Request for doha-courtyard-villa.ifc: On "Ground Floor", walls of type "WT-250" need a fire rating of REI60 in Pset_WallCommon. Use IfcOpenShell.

First a look at what the model holds.

```python
import ifcopenshell
import ifcopenshell.util.element

model = ifcopenshell.open("doha-courtyard-villa.ifc")
print(model.schema)
storey = next(s for s in model.by_type("IfcBuildingStorey") if s.Name == "Ground Floor")
walls = [e for e in ifcopenshell.util.element.get_decomposition(storey) if e.is_a("IfcWall")]
seen = {}
for e in walls:
    element_type = ifcopenshell.util.element.get_type(e)
    key = (element_type.Name if element_type != e and element_type else None, ifcopenshell.util.element.get_pset(e, "Pset_WallCommon", "FireRating"))
    seen[key] = seen.get(key, 0) + 1
for (name, value), count in sorted(seen.items(), key=str):
    print(count, "x", name, "|", value)
```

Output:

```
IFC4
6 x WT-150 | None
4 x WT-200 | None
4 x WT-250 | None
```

```python
import ifcopenshell
import ifcopenshell.api.pset
import ifcopenshell.util.element

model = ifcopenshell.open("doha-courtyard-villa.ifc")

storey = next(s for s in model.by_type("IfcBuildingStorey") if s.Name == "Ground Floor")
walls = [e for e in ifcopenshell.util.element.get_decomposition(storey) if e.is_a("IfcWall")]

count = 0
for e in walls:
    element_type = ifcopenshell.util.element.get_type(e)
    if element_type in (None, e) or element_type.Name != "WT-250":
        continue
    # add_pset returns the element's existing set when there is one.
    pset = ifcopenshell.api.pset.add_pset(model, product=e, name="Pset_WallCommon")
    ifcopenshell.api.pset.edit_pset(model, pset=pset, properties={"FireRating": "REI60"})
    count += 1

print(count, "walls updated")

model.write("doha-courtyard-villa_v2.ifc")
```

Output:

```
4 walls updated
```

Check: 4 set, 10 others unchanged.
